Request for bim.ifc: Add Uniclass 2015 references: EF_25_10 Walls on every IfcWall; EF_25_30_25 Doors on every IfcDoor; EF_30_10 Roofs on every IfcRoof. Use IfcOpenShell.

First a look at what the model holds.

```python
import ifcopenshell

model = ifcopenshell.open("bim.ifc")
print(model.schema)
print("classifications:", [c.Name for c in model.by_type("IfcClassification")])
for ifc_class in ("IfcDoor", "IfcRoof", "IfcStair", "IfcWall", "IfcWindow"):
    print(ifc_class, len(model.by_type(ifc_class)))
```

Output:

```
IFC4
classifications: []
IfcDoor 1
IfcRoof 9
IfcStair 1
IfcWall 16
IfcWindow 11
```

```python
import ifcopenshell
import ifcopenshell.api.classification

model = ifcopenshell.open("bim.ifc")

system = ifcopenshell.api.classification.add_classification(model, classification="Uniclass 2015")

codes = {
    "IfcWall": ("EF_25_10", "Walls"),
    "IfcDoor": ("EF_25_30_25", "Doors"),
    "IfcRoof": ("EF_30_10", "Roofs"),
}
for ifc_class, (code, name) in codes.items():
    products = model.by_type(ifc_class)
    ifcopenshell.api.classification.add_reference(
        model, products=products, classification=system, identification=code, name=name
    )
    print(code, len(products))

model.write("bim_v2.ifc")
```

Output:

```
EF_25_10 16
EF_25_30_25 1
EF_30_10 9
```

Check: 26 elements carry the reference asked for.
